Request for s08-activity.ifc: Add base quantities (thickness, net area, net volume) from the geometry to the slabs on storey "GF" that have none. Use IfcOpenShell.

First a look at what the model holds.

```python
import ifcopenshell
import ifcopenshell.util.element
import ifcopenshell.util.unit

model = ifcopenshell.open("s08-activity.ifc")
print(model.schema)
for unit_type in ("LENGTHUNIT", "AREAUNIT", "VOLUMEUNIT"):
    print(unit_type, ifcopenshell.util.unit.calculate_unit_scale(model, unit_type))
storey = next(s for s in model.by_type("IfcBuildingStorey") if s.Name == "GF")
slabs = [e for e in ifcopenshell.util.element.get_decomposition(storey) if e.is_a("IfcSlab")]
for e in sorted(slabs, key=lambda e: e.id()):
    print(e.id(), e.is_a(), e.Name, list(ifcopenshell.util.element.get_psets(e, qtos_only=True)), sep=" | ")
```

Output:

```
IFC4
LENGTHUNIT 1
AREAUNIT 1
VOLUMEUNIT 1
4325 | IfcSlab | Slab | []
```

```python
import ifcopenshell
import ifcopenshell.api.pset
import ifcopenshell.geom
import ifcopenshell.util.element
import ifcopenshell.util.shape
import ifcopenshell.util.unit

model = ifcopenshell.open("s08-activity.ifc")
unit_scale = ifcopenshell.util.unit.calculate_unit_scale(model)
area_scale = ifcopenshell.util.unit.calculate_unit_scale(model, "AREAUNIT")
volume_scale = ifcopenshell.util.unit.calculate_unit_scale(model, "VOLUMEUNIT")
settings = ifcopenshell.geom.settings()

storey = next(s for s in model.by_type("IfcBuildingStorey") if s.Name == "GF")
slabs = [e for e in ifcopenshell.util.element.get_decomposition(storey) if e.is_a("IfcSlab")]

for e in sorted(slabs, key=lambda e: e.id()):
    if ifcopenshell.util.element.get_psets(e, qtos_only=True, should_inherit=False):
        continue
    # Geometry comes back in metres, in the element's own axes.
    shape = ifcopenshell.geom.create_shape(settings, e)
    values = {
        "Width": ifcopenshell.util.shape.get_z(shape.geometry) / unit_scale,
        "NetArea": ifcopenshell.util.shape.get_footprint_area(shape.geometry) / area_scale,
        "NetVolume": ifcopenshell.util.shape.get_volume(shape.geometry) / volume_scale,
    }
    qto = ifcopenshell.api.pset.add_qto(model, product=e, name="Qto_SlabBaseQuantities")
    ifcopenshell.api.pset.edit_qto(model, qto=qto, properties=values)
    print(e.id(), {k: round(v, 3) for k, v in values.items()})

model.write("s08-activity_updated.ifc")
```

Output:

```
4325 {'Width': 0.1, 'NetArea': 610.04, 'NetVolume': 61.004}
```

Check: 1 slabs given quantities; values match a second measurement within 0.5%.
